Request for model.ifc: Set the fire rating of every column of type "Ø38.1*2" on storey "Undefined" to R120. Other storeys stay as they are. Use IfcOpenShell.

First a look at what the model holds.

```python
import ifcopenshell
import ifcopenshell.util.element

model = ifcopenshell.open("model.ifc")
print(model.schema)
storey = next(s for s in model.by_type("IfcBuildingStorey") if s.Name == "Undefined")
columns = [e for e in ifcopenshell.util.element.get_decomposition(storey) if e.is_a("IfcColumn")]
seen = {}
for e in columns:
    element_type = ifcopenshell.util.element.get_type(e)
    key = (element_type.Name if element_type != e and element_type else None, ifcopenshell.util.element.get_pset(e, "Pset_ColumnCommon", "FireRating"))
    seen[key] = seen.get(key, 0) + 1
for (name, value), count in sorted(seen.items(), key=str):
    print(count, "x", name, "|", value)
```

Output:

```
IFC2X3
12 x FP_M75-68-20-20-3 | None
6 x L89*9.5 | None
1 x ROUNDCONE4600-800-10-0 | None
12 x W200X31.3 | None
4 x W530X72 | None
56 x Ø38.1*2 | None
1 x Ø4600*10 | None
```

```python
import ifcopenshell
import ifcopenshell.api.pset
import ifcopenshell.util.element

model = ifcopenshell.open("model.ifc")

storey = next(s for s in model.by_type("IfcBuildingStorey") if s.Name == "Undefined")
columns = [e for e in ifcopenshell.util.element.get_decomposition(storey) if e.is_a("IfcColumn")]

count = 0
for e in columns:
    element_type = ifcopenshell.util.element.get_type(e)
    if element_type in (None, e) or element_type.Name != "Ø38.1*2":
        continue
    # add_pset returns the element's existing set when there is one.
    pset = ifcopenshell.api.pset.add_pset(model, product=e, name="Pset_ColumnCommon")
    ifcopenshell.api.pset.edit_pset(model, pset=pset, properties={"FireRating": "R120"})
    count += 1

print(count, "columns updated")

model.write("model_updated.ifc")
```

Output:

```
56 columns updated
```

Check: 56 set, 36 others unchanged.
